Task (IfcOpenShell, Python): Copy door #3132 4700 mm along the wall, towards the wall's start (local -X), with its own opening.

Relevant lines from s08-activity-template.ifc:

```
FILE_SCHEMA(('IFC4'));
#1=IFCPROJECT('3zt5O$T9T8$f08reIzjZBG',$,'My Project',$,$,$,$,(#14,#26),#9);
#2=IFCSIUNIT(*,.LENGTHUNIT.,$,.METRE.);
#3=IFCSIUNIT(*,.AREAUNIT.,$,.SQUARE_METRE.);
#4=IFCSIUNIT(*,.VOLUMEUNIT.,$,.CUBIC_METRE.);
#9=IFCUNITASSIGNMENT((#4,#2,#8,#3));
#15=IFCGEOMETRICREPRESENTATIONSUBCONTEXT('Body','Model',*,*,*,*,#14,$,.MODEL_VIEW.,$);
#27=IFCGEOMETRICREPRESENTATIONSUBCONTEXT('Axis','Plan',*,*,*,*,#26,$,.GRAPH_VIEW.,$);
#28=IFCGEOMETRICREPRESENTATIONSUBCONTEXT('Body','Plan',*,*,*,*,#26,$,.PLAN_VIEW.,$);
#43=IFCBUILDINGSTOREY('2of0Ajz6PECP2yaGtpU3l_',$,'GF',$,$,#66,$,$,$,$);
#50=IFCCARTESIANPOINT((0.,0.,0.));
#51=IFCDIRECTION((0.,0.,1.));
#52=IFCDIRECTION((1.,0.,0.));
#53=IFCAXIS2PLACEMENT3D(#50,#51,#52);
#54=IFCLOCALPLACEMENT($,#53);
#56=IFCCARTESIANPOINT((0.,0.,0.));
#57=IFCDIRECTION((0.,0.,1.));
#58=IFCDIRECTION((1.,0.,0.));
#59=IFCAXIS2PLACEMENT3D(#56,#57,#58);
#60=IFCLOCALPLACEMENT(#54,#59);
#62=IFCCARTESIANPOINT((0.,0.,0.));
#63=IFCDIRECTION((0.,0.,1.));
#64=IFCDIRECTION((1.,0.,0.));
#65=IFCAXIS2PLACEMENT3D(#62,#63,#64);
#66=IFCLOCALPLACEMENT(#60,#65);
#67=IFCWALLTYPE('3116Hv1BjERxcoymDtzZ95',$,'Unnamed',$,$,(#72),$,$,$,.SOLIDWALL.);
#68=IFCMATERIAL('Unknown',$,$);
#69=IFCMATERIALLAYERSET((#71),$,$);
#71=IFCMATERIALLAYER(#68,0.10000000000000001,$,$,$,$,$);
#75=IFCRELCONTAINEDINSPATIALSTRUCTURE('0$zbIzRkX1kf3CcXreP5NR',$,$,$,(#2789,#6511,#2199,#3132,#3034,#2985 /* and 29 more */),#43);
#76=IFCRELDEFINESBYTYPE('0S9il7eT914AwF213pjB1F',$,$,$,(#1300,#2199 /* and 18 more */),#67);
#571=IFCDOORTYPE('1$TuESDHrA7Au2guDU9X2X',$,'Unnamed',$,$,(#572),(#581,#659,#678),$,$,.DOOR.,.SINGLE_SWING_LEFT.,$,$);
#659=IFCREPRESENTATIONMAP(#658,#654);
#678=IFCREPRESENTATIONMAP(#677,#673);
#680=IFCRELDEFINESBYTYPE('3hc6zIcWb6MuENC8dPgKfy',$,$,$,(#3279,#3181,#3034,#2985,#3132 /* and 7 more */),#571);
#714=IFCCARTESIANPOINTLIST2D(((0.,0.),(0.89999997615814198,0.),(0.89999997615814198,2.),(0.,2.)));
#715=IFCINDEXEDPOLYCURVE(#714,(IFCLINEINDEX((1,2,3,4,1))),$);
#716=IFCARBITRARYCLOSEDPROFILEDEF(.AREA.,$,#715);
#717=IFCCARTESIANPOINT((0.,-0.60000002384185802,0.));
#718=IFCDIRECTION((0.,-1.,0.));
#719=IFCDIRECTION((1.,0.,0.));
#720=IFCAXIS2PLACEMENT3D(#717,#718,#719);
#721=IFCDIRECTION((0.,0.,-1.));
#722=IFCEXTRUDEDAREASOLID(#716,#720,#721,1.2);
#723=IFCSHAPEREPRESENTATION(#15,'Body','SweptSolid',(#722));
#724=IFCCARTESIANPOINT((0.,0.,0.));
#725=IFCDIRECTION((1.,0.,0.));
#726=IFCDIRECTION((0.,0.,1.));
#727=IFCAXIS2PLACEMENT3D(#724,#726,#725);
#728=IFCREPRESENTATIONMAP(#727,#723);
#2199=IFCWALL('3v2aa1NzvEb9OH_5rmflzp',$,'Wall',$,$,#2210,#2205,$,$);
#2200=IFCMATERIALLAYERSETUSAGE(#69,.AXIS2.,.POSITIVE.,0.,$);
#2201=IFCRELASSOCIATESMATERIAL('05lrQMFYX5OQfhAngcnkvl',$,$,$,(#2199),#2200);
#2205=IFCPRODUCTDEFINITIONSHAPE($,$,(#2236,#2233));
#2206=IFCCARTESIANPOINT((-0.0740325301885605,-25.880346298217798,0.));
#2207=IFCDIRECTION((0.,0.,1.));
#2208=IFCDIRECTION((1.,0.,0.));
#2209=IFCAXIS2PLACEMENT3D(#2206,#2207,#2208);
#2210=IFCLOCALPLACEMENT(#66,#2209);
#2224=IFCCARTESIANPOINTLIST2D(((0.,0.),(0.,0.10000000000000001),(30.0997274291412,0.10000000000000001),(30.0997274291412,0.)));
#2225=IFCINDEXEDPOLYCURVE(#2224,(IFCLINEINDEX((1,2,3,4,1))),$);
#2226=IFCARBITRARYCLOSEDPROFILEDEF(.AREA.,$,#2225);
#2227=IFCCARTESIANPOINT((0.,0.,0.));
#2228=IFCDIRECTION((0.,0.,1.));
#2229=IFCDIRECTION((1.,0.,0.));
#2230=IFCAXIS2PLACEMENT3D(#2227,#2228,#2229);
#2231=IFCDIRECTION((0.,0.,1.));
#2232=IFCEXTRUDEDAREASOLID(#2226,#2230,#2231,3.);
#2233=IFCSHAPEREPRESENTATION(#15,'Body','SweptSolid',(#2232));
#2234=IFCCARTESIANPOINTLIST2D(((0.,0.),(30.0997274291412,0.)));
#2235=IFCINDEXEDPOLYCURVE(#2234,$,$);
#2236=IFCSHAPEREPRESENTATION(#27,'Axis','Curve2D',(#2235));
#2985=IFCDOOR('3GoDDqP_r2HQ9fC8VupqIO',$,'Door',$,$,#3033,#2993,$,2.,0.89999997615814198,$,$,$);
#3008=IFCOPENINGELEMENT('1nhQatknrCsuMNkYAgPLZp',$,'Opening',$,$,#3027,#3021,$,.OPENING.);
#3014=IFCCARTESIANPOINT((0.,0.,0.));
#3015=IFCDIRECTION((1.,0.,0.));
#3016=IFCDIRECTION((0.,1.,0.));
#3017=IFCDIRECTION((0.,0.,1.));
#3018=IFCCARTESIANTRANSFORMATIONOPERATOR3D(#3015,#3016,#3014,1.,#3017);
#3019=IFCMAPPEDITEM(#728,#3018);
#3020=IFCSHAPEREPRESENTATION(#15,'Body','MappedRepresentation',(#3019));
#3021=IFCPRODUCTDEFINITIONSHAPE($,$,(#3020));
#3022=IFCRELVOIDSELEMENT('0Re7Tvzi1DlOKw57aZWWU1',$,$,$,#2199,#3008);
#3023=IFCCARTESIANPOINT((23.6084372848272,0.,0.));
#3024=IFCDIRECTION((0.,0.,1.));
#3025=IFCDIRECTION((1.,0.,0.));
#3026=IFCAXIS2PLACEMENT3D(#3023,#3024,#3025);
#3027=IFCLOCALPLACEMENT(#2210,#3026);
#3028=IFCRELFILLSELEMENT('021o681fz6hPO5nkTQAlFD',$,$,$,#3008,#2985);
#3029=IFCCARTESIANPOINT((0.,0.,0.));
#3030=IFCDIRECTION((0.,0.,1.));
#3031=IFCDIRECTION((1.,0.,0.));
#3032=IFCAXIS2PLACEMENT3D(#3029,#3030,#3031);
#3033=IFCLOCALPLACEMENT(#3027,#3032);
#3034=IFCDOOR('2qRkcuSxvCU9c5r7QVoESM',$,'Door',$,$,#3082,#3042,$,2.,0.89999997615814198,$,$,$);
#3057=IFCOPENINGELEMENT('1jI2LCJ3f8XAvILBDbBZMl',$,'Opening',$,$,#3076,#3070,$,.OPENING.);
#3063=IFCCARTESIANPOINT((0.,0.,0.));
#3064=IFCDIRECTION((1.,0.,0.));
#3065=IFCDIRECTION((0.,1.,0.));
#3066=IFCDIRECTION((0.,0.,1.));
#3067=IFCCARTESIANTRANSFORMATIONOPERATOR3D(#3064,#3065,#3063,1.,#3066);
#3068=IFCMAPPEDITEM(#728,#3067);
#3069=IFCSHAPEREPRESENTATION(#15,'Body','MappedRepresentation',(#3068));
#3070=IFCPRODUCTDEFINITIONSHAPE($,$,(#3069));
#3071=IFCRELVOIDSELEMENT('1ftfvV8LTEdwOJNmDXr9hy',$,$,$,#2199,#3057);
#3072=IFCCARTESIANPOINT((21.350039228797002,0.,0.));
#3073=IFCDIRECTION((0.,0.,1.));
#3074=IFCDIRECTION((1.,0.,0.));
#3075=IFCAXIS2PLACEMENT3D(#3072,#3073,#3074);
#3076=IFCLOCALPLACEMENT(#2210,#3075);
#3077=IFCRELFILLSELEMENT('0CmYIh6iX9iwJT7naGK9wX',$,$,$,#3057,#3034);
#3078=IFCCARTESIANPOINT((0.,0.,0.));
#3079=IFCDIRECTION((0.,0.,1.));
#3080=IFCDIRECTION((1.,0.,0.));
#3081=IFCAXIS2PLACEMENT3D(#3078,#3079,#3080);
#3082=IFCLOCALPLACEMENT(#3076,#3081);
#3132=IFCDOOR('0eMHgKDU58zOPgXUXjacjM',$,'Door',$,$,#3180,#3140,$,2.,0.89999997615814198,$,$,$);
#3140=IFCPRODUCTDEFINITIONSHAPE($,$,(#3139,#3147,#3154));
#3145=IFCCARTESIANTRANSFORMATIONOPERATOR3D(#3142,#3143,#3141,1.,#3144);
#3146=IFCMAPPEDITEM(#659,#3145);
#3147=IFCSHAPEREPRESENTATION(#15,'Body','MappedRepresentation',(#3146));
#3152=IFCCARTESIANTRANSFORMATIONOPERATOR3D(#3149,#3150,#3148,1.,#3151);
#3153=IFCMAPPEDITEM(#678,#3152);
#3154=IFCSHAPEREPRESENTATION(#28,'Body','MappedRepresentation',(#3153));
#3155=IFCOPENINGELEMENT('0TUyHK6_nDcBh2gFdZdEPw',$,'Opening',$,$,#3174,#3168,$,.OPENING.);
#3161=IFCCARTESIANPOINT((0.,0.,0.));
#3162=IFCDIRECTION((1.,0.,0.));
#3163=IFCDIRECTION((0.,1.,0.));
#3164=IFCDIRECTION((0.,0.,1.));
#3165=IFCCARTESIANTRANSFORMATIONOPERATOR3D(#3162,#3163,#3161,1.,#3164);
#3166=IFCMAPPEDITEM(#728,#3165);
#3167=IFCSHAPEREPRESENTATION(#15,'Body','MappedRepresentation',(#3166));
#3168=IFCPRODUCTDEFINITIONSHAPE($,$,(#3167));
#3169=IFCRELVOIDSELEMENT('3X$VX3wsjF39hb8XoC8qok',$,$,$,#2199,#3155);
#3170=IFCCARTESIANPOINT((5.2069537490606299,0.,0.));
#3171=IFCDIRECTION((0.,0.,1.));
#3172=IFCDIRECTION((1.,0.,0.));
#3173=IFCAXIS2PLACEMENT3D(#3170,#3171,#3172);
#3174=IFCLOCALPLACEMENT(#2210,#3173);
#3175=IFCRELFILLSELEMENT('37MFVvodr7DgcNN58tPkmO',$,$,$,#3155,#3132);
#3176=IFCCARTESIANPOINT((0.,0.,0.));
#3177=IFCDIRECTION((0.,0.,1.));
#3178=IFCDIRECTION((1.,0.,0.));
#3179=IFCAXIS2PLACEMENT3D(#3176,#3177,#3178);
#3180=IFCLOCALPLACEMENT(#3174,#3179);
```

```python
import ifcopenshell
import ifcopenshell.api.feature
import ifcopenshell.api.geometry
import ifcopenshell.api.root
import ifcopenshell.geom
import ifcopenshell.util.element
import ifcopenshell.util.placement
import ifcopenshell.util.shape
import ifcopenshell.util.unit

model = ifcopenshell.open("s08-activity-template.ifc")
unit_scale = ifcopenshell.util.unit.calculate_unit_scale(model)
settings = ifcopenshell.geom.settings()


def volume(element):
    """Net volume in cubic metres, openings subtracted."""
    shape = ifcopenshell.geom.create_shape(settings, element)
    return ifcopenshell.util.shape.get_volume(shape.geometry)


door = model.by_id(3132)
opening = door.FillsVoids[0].RelatingOpeningElement
wall = opening.VoidsElements[0].RelatingBuildingElement
before = volume(wall)
shift = ifcopenshell.util.placement.get_local_placement(wall.ObjectPlacement)[:3, 0] * -4.7 / unit_scale

# copy_class copies the void relationship, type, container and properties, but no geometry.
new_opening = ifcopenshell.api.root.copy_class(model, product=opening)
new_opening.Representation = ifcopenshell.util.element.copy_deep(
    model, opening.Representation, exclude=["IfcGeometricRepresentationContext", "IfcRepresentationMap"]
)
new_door = ifcopenshell.api.root.copy_class(model, product=door)
new_door.Representation = ifcopenshell.util.element.copy_deep(
    model, door.Representation, exclude=["IfcGeometricRepresentationContext", "IfcRepresentationMap"]
)
ifcopenshell.api.feature.add_filling(model, opening=new_opening, element=new_door)

for old, new in ((opening, new_opening), (door, new_door)):
    matrix = ifcopenshell.util.placement.get_local_placement(old.ObjectPlacement)
    matrix[:3, 3] += shift
    ifcopenshell.api.geometry.edit_object_placement(model, product=new, matrix=matrix, is_si=False)

after = volume(wall)

print(f"wall volume {before:.3f} -> {after:.3f} m3")

model.write("s08-activity-template_updated.ifc")
```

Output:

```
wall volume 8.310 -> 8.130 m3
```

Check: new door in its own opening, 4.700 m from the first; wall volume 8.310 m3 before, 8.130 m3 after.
